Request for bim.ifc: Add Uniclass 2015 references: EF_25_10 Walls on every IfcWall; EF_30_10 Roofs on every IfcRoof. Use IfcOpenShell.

First a look at what the model holds.

```python
import ifcopenshell

model = ifcopenshell.open("bim.ifc")
print(model.schema)
print("classifications:", [c.Name for c in model.by_type("IfcClassification")])
for ifc_class in ("IfcDoor", "IfcRoof", "IfcStair", "IfcWall", "IfcWindow"):
    print(ifc_class, len(model.by_type(ifc_class)))
```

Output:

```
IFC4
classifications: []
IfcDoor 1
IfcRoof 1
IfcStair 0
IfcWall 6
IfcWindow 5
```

```python
import ifcopenshell
import ifcopenshell.api.classification

model = ifcopenshell.open("bim.ifc")

system = ifcopenshell.api.classification.add_classification(model, classification="Uniclass 2015")

codes = {
    "IfcWall": ("EF_25_10", "Walls"),
    "IfcRoof": ("EF_30_10", "Roofs"),
}
for ifc_class, (code, name) in codes.items():
    products = model.by_type(ifc_class)
    ifcopenshell.api.classification.add_reference(
        model, products=products, classification=system, identification=code, name=name
    )
    print(code, len(products))

model.write("bim_rev.ifc")
```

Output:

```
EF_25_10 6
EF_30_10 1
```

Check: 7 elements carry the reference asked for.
